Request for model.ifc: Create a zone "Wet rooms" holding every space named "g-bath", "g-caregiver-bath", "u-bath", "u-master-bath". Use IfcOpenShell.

First a look at what the model holds.

```python
import ifcopenshell

model = ifcopenshell.open("model.ifc")
print(model.schema)
seen = {}
for space in model.by_type("IfcSpace"):
    seen[space.LongName] = seen.get(space.LongName, 0) + 1
for name, count in sorted(seen.items(), key=str):
    print(count, "x", name)
print("zones:", [z.Name for z in model.by_type("IfcZone")][:20])
```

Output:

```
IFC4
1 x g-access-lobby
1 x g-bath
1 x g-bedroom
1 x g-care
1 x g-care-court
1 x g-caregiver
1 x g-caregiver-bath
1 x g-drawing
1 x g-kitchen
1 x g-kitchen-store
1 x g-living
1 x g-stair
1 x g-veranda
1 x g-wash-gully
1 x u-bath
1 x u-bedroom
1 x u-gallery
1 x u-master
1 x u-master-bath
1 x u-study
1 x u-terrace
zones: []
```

```python
import ifcopenshell
import ifcopenshell.api.group
import ifcopenshell.api.root

model = ifcopenshell.open("model.ifc")

names = {"g-bath", "g-caregiver-bath", "u-bath", "u-master-bath"}
spaces = [s for s in model.by_type("IfcSpace") if s.LongName in names]

zone = ifcopenshell.api.root.create_entity(model, ifc_class="IfcZone", name="Wet rooms")
ifcopenshell.api.group.assign_group(model, products=spaces, group=zone)
print(len(spaces), "spaces in", zone.Name)

model.write("model_rev.ifc")
```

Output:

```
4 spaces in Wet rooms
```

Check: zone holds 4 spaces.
